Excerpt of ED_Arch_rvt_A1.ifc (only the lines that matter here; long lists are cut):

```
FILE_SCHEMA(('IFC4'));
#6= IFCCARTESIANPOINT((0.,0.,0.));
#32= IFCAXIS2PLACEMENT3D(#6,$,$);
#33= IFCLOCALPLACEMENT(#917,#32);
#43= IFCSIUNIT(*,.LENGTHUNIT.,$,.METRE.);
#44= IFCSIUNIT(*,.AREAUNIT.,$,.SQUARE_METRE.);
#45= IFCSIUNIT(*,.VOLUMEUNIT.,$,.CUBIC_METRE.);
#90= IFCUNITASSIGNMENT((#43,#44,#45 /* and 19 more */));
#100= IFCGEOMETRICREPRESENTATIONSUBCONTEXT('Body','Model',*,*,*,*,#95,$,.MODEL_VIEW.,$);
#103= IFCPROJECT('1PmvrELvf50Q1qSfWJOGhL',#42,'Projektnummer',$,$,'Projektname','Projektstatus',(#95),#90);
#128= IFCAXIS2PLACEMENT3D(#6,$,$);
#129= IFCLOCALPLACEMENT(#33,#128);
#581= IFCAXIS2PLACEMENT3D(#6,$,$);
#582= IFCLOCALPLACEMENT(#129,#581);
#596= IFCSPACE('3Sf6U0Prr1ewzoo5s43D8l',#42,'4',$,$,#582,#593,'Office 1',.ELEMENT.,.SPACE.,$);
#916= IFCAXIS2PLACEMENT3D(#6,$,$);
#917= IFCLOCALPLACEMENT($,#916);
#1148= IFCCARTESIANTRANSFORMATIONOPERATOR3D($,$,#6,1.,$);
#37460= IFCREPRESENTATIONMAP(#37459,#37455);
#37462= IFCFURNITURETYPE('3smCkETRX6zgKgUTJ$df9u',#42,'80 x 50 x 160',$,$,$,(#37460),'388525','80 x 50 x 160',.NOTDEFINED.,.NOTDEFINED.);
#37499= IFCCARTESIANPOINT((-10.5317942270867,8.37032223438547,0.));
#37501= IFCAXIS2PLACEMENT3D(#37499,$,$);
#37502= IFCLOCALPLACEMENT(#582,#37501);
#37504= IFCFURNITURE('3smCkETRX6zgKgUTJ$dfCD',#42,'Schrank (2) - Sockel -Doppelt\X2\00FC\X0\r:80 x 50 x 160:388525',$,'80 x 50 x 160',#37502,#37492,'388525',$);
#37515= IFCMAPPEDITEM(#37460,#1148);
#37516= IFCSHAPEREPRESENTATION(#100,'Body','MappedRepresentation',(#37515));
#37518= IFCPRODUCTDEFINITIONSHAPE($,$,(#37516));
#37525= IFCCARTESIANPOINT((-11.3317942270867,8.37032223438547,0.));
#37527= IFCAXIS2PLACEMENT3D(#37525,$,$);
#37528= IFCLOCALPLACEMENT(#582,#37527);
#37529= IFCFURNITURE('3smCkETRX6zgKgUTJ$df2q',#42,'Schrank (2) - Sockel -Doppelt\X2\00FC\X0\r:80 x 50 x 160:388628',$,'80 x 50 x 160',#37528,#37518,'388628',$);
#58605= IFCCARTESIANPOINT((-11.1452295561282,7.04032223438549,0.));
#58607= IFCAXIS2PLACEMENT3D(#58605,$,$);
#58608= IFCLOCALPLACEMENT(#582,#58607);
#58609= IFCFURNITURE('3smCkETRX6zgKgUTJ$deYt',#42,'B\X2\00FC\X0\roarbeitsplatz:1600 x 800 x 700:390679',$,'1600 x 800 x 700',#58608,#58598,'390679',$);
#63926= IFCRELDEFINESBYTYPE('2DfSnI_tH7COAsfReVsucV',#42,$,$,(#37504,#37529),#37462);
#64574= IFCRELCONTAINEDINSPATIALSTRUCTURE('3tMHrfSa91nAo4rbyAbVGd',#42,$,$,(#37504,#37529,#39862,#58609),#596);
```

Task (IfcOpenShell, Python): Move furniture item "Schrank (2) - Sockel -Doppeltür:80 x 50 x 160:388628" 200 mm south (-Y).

```python
import ifcopenshell
import ifcopenshell.api.geometry
import ifcopenshell.util.placement

model = ifcopenshell.open("ED_Arch_rvt_A1.ifc")

item = model.by_guid("3smCkETRX6zgKgUTJ$df2q")
matrix = ifcopenshell.util.placement.get_local_placement(item.ObjectPlacement)
matrix[1, 3] -= 0.2
ifcopenshell.api.geometry.edit_object_placement(model, product=item, matrix=matrix, is_si=False)

print(ifcopenshell.util.placement.get_local_placement(item.ObjectPlacement).round(3) + 0.0)

model.write("ED_Arch_rvt_A1-out.ifc")
```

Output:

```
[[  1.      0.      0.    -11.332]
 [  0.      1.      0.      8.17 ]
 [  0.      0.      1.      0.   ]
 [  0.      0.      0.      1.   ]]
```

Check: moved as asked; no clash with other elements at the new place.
